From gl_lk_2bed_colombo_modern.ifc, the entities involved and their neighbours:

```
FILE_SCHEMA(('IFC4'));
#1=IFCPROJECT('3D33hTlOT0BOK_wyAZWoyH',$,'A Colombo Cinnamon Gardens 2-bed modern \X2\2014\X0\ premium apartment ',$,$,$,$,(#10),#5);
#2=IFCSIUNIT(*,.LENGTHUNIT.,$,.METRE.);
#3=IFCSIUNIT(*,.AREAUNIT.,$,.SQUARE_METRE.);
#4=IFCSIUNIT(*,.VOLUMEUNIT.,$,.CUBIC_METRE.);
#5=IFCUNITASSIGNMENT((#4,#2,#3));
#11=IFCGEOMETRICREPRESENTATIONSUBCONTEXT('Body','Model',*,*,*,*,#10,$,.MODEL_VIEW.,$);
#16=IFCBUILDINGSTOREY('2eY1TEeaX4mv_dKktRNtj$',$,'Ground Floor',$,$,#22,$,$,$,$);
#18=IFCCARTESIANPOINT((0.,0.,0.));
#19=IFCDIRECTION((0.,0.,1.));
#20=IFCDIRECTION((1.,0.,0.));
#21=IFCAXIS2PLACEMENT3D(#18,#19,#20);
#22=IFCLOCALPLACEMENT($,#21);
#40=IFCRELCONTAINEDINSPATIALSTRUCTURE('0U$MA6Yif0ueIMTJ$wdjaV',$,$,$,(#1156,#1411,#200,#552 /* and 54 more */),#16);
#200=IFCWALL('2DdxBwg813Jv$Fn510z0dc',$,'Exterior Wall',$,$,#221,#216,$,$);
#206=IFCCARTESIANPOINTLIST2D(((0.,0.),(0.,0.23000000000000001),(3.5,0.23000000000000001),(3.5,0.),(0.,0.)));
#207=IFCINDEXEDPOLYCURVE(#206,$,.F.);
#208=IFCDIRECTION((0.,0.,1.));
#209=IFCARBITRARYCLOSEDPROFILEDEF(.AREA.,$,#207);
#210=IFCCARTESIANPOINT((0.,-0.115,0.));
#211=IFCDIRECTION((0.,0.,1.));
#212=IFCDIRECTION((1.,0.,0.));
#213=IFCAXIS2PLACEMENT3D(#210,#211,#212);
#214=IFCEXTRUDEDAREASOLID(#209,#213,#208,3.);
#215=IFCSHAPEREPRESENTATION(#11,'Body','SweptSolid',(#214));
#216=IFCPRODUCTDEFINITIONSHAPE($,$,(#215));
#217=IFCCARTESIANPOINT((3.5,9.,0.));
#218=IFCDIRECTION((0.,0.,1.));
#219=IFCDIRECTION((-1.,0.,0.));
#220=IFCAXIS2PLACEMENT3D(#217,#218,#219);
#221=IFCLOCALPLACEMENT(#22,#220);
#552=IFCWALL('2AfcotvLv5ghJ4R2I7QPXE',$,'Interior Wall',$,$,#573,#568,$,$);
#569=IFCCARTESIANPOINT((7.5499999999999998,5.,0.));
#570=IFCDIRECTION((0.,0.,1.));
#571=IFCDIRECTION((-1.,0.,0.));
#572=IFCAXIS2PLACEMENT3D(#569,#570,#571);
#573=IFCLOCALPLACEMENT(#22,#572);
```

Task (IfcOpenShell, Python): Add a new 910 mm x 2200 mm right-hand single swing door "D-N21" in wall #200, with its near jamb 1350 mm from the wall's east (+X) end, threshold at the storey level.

```python
import numpy as np
import ifcopenshell
import ifcopenshell.api.feature
import ifcopenshell.api.geometry
import ifcopenshell.api.root
import ifcopenshell.api.spatial
import ifcopenshell.geom
import ifcopenshell.util.element
import ifcopenshell.util.placement
import ifcopenshell.util.representation
import ifcopenshell.util.shape
import ifcopenshell.util.unit

model = ifcopenshell.open("gl_lk_2bed_colombo_modern.ifc")
unit_scale = ifcopenshell.util.unit.calculate_unit_scale(model)
settings = ifcopenshell.geom.settings()


def volume(element):
    """Net volume in cubic metres, openings subtracted."""
    shape = ifcopenshell.geom.create_shape(settings, element)
    return ifcopenshell.util.shape.get_volume(shape.geometry)


wall = model.by_id(200)
storey = ifcopenshell.util.element.get_container(wall, ifc_class="IfcBuildingStorey")
context = ifcopenshell.util.representation.get_context(model, "Model", "Body", "MODEL_VIEW")
before = volume(wall)

width, height, from_end, sill = 0.91, 2.2, 1.35, 0.0  # metres

# The wall runs along its own X axis, and the end named is its -X end.
wall_shape = ifcopenshell.geom.create_shape(settings, wall)
x, y, z = ifcopenshell.util.shape.get_vertices(wall_shape.geometry).T
start = x.min() + from_end
face, thickness = float(y.min()), float(y.max() - y.min())
wall_matrix = ifcopenshell.util.placement.get_local_placement(wall.ObjectPlacement)
level = ifcopenshell.util.placement.get_local_placement(storey.ObjectPlacement)[2, 3]


def in_wall(x, y):
    """Placement at x, y metres in the wall's axes, at sill height."""
    matrix = wall_matrix.copy()
    matrix[:, 3] = wall_matrix @ np.array([x / unit_scale, y / unit_scale, 0.0, 1.0])
    matrix[2, 3] = level + sill / unit_scale
    return matrix


# Opening: a box that overshoots both wall faces by 50 mm.
opening = ifcopenshell.api.root.create_entity(model, ifc_class="IfcOpeningElement", predefined_type="OPENING")
box = ifcopenshell.api.geometry.add_wall_representation(
    model, context=context, length=width, height=height, thickness=thickness + 0.1
)
ifcopenshell.api.geometry.assign_representation(model, product=opening, representation=box)
ifcopenshell.api.geometry.edit_object_placement(model, product=opening, matrix=in_wall(start, face - 0.05), is_si=False)
ifcopenshell.api.feature.add_feature(model, feature=opening, element=wall)

door = ifcopenshell.api.root.create_entity(model, ifc_class="IfcDoor", name="D-N21", predefined_type="DOOR")
door.OverallWidth, door.OverallHeight = width / unit_scale, height / unit_scale
door.OperationType = "SINGLE_SWING_RIGHT"
body = ifcopenshell.api.geometry.add_door_representation(
    model,
    context=context,
    overall_width=door.OverallWidth,
    overall_height=door.OverallHeight,
    operation_type="SINGLE_SWING_RIGHT",
    lining_properties={"LiningDepth": thickness / unit_scale, "ThresholdDepth": thickness / unit_scale},
)
ifcopenshell.api.geometry.assign_representation(model, product=door, representation=body)
ifcopenshell.api.spatial.assign_container(model, products=[door], relating_structure=storey)
ifcopenshell.api.feature.add_filling(model, opening=opening, element=door)

# The lining spans the wall, so the door starts at the wall face.
ifcopenshell.api.geometry.edit_object_placement(model, product=door, matrix=in_wall(start, face), is_si=False)

after = volume(wall)

print(f"wall volume {before:.3f} -> {after:.3f} m3")

model.write("gl_lk_2bed_colombo_modern_edited.ifc")
```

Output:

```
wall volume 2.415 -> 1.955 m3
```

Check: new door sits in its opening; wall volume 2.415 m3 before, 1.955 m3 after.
